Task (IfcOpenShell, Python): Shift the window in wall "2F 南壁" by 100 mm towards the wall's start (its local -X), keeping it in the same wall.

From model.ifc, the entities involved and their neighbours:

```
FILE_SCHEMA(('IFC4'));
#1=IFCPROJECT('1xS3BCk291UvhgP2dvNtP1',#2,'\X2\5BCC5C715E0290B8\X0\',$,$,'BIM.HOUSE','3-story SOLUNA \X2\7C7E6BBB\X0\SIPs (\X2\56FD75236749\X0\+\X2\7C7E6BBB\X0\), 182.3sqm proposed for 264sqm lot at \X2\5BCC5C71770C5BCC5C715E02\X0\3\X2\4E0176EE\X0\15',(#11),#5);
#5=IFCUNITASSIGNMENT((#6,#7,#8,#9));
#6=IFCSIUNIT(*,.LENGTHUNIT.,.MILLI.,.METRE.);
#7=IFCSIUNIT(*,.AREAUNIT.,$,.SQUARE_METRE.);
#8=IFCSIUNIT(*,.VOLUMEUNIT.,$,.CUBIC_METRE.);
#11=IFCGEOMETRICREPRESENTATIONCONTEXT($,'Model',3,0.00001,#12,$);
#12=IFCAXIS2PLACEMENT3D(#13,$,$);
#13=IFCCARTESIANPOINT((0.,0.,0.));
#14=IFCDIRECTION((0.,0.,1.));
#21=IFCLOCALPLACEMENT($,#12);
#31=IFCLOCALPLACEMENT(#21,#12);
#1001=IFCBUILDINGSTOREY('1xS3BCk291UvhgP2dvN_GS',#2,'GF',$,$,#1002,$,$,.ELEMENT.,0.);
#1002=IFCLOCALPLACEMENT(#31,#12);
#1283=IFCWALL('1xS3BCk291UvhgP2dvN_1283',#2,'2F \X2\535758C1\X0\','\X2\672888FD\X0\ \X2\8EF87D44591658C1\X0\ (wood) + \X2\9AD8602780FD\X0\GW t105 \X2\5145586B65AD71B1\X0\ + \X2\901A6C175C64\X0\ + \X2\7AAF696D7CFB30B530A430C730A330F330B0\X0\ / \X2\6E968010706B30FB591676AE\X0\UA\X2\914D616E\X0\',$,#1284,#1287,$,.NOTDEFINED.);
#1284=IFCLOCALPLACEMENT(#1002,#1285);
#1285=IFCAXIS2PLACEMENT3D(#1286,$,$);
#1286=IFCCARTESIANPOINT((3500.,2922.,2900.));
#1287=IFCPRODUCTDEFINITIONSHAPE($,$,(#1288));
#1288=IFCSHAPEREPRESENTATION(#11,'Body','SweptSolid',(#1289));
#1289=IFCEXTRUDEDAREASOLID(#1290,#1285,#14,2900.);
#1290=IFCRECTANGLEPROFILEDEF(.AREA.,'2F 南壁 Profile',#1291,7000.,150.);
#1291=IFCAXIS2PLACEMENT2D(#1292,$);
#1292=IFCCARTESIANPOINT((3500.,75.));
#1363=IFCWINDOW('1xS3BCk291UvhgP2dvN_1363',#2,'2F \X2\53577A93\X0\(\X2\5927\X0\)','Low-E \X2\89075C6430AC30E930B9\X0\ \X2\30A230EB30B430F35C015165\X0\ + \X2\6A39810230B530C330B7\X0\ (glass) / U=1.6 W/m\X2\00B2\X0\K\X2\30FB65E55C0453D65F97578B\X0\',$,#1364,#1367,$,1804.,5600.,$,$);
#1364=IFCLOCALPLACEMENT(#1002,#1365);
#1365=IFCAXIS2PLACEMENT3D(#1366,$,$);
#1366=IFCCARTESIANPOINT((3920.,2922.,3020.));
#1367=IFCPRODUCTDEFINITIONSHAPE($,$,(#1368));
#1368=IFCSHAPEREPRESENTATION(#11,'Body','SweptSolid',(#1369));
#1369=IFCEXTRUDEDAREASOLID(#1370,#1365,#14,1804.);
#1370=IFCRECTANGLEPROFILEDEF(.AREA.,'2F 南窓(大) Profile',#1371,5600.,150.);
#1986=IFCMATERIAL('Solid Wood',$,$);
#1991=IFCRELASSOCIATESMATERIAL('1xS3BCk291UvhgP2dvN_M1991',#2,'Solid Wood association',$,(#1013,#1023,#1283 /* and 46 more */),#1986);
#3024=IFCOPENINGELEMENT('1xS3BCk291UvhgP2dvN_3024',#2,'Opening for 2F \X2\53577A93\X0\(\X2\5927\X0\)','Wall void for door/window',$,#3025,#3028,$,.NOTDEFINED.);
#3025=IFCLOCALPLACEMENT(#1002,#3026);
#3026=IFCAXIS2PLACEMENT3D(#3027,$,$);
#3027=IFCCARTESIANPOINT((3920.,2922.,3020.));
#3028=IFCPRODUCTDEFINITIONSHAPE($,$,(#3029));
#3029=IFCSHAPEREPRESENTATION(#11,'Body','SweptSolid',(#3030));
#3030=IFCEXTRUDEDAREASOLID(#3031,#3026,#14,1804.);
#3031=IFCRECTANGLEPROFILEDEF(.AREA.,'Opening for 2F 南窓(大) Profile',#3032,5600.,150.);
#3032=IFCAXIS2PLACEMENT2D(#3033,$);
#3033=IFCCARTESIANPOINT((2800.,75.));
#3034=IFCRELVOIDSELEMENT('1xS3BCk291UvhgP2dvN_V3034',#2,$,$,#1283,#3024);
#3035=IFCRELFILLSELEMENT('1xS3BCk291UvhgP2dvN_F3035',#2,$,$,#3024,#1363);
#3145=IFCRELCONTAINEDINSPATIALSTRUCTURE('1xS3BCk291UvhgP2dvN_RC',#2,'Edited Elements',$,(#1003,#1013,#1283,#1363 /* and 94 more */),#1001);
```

```python
import ifcopenshell
import ifcopenshell.api.geometry
import ifcopenshell.util.placement

model = ifcopenshell.open("model.ifc")

window = model.by_guid("1xS3BCk291UvhgP2dvN_1363")
opening = window.FillsVoids[0].RelatingOpeningElement
wall = opening.VoidsElements[0].RelatingBuildingElement

wall_matrix = ifcopenshell.util.placement.get_local_placement(wall.ObjectPlacement)
shift = wall_matrix[:3, 0] * -100.0
before = ifcopenshell.util.placement.get_local_placement(window.ObjectPlacement)[:3, 3].copy()

# The window is not placed relative to its opening, so move both.
for product in (opening, window):
    matrix = ifcopenshell.util.placement.get_local_placement(product.ObjectPlacement)
    matrix[:3, 3] += shift
    ifcopenshell.api.geometry.edit_object_placement(model, product=product, matrix=matrix, is_si=False)

after = ifcopenshell.util.placement.get_local_placement(window.ObjectPlacement)[:3, 3]
print("window moved by", (after - before).round(3) + 0.0)

model.write("model_v2.ifc")
```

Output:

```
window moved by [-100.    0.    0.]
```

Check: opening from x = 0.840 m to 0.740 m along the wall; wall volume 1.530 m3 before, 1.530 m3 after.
